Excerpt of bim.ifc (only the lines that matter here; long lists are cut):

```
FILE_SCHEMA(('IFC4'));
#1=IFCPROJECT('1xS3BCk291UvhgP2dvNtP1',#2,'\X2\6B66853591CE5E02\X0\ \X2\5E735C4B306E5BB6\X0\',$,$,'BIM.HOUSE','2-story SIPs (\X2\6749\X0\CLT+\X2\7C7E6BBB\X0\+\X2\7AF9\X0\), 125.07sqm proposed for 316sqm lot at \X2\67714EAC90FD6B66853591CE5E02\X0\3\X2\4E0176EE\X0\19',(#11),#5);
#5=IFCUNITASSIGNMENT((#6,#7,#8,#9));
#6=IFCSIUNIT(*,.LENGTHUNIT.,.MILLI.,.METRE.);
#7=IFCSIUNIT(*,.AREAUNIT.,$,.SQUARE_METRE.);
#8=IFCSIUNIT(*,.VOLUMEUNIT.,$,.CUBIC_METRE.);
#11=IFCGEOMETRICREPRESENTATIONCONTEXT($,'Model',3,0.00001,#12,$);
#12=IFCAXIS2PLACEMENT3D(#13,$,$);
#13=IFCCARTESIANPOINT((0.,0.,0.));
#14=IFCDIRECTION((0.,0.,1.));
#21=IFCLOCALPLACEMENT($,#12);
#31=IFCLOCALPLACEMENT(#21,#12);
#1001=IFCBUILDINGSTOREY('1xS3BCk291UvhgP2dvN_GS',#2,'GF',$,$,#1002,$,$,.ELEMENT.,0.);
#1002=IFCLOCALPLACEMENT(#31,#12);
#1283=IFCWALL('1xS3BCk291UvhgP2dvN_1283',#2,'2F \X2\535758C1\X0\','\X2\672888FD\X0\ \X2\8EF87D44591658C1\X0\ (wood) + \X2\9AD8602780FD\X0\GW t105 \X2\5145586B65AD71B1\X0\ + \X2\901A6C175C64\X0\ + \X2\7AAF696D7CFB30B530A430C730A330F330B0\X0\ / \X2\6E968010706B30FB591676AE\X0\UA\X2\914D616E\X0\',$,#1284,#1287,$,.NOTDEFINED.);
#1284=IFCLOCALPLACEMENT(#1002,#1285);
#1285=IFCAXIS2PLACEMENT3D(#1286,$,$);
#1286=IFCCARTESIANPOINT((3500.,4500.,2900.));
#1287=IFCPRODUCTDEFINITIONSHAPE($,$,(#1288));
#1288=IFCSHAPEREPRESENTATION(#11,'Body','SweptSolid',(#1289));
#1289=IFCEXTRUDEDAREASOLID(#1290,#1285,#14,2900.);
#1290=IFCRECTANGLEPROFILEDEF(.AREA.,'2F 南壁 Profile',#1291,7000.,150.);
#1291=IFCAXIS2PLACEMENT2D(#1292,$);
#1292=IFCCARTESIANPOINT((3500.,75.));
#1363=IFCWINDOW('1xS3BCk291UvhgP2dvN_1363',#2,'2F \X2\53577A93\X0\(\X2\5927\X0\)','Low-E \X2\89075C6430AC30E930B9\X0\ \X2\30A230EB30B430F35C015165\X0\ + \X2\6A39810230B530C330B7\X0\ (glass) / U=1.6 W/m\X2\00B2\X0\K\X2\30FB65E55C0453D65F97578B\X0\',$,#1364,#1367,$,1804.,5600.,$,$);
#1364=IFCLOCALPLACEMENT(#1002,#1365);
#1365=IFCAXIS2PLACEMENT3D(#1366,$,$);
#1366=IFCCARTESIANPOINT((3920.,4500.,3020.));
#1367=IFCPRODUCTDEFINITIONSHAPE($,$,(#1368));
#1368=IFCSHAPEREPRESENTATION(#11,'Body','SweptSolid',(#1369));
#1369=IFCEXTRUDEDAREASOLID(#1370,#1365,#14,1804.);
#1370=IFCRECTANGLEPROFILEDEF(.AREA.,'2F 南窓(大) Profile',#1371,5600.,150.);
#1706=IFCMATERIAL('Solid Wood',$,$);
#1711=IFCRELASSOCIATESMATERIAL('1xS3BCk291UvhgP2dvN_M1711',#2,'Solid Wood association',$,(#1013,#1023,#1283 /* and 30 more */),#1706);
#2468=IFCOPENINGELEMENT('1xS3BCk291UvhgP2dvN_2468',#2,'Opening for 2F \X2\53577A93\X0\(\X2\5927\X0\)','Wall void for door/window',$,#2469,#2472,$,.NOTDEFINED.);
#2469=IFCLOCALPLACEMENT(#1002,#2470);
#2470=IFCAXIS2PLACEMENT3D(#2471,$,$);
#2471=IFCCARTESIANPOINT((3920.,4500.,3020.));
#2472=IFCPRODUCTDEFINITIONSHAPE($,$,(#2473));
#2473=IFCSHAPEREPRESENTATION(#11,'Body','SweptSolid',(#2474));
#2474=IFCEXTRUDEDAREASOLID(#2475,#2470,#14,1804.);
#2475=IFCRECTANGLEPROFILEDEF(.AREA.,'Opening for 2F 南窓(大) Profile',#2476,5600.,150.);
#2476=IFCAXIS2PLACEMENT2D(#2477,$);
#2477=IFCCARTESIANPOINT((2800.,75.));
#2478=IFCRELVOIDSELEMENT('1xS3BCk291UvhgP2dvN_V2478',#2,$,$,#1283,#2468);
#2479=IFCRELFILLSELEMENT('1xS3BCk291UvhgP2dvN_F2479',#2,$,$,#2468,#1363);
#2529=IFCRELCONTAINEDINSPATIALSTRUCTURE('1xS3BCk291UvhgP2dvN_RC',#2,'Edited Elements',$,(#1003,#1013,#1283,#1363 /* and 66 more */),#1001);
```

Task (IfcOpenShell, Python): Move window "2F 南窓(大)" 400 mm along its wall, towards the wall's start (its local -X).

```python
import ifcopenshell
import ifcopenshell.api.geometry
import ifcopenshell.util.placement
import ifcopenshell.util.unit

model = ifcopenshell.open("bim.ifc")
unit_scale = ifcopenshell.util.unit.calculate_unit_scale(model)

window = model.by_guid("1xS3BCk291UvhgP2dvN_1363")
opening = window.FillsVoids[0].RelatingOpeningElement
wall = opening.VoidsElements[0].RelatingBuildingElement

wall_matrix = ifcopenshell.util.placement.get_local_placement(wall.ObjectPlacement)
shift = wall_matrix[:3, 0] * -0.4 / unit_scale
before = ifcopenshell.util.placement.get_local_placement(window.ObjectPlacement)[:3, 3].copy()

# The window is not placed relative to its opening, so move both.
for product in (opening, window):
    matrix = ifcopenshell.util.placement.get_local_placement(product.ObjectPlacement)
    matrix[:3, 3] += shift
    ifcopenshell.api.geometry.edit_object_placement(model, product=product, matrix=matrix, is_si=False)

after = ifcopenshell.util.placement.get_local_placement(window.ObjectPlacement)[:3, 3]
print("window moved by", (after - before).round(3) + 0.0)

model.write("bim_v2.ifc")
```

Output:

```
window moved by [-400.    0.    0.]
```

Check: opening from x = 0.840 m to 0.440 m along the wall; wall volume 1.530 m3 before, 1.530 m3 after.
